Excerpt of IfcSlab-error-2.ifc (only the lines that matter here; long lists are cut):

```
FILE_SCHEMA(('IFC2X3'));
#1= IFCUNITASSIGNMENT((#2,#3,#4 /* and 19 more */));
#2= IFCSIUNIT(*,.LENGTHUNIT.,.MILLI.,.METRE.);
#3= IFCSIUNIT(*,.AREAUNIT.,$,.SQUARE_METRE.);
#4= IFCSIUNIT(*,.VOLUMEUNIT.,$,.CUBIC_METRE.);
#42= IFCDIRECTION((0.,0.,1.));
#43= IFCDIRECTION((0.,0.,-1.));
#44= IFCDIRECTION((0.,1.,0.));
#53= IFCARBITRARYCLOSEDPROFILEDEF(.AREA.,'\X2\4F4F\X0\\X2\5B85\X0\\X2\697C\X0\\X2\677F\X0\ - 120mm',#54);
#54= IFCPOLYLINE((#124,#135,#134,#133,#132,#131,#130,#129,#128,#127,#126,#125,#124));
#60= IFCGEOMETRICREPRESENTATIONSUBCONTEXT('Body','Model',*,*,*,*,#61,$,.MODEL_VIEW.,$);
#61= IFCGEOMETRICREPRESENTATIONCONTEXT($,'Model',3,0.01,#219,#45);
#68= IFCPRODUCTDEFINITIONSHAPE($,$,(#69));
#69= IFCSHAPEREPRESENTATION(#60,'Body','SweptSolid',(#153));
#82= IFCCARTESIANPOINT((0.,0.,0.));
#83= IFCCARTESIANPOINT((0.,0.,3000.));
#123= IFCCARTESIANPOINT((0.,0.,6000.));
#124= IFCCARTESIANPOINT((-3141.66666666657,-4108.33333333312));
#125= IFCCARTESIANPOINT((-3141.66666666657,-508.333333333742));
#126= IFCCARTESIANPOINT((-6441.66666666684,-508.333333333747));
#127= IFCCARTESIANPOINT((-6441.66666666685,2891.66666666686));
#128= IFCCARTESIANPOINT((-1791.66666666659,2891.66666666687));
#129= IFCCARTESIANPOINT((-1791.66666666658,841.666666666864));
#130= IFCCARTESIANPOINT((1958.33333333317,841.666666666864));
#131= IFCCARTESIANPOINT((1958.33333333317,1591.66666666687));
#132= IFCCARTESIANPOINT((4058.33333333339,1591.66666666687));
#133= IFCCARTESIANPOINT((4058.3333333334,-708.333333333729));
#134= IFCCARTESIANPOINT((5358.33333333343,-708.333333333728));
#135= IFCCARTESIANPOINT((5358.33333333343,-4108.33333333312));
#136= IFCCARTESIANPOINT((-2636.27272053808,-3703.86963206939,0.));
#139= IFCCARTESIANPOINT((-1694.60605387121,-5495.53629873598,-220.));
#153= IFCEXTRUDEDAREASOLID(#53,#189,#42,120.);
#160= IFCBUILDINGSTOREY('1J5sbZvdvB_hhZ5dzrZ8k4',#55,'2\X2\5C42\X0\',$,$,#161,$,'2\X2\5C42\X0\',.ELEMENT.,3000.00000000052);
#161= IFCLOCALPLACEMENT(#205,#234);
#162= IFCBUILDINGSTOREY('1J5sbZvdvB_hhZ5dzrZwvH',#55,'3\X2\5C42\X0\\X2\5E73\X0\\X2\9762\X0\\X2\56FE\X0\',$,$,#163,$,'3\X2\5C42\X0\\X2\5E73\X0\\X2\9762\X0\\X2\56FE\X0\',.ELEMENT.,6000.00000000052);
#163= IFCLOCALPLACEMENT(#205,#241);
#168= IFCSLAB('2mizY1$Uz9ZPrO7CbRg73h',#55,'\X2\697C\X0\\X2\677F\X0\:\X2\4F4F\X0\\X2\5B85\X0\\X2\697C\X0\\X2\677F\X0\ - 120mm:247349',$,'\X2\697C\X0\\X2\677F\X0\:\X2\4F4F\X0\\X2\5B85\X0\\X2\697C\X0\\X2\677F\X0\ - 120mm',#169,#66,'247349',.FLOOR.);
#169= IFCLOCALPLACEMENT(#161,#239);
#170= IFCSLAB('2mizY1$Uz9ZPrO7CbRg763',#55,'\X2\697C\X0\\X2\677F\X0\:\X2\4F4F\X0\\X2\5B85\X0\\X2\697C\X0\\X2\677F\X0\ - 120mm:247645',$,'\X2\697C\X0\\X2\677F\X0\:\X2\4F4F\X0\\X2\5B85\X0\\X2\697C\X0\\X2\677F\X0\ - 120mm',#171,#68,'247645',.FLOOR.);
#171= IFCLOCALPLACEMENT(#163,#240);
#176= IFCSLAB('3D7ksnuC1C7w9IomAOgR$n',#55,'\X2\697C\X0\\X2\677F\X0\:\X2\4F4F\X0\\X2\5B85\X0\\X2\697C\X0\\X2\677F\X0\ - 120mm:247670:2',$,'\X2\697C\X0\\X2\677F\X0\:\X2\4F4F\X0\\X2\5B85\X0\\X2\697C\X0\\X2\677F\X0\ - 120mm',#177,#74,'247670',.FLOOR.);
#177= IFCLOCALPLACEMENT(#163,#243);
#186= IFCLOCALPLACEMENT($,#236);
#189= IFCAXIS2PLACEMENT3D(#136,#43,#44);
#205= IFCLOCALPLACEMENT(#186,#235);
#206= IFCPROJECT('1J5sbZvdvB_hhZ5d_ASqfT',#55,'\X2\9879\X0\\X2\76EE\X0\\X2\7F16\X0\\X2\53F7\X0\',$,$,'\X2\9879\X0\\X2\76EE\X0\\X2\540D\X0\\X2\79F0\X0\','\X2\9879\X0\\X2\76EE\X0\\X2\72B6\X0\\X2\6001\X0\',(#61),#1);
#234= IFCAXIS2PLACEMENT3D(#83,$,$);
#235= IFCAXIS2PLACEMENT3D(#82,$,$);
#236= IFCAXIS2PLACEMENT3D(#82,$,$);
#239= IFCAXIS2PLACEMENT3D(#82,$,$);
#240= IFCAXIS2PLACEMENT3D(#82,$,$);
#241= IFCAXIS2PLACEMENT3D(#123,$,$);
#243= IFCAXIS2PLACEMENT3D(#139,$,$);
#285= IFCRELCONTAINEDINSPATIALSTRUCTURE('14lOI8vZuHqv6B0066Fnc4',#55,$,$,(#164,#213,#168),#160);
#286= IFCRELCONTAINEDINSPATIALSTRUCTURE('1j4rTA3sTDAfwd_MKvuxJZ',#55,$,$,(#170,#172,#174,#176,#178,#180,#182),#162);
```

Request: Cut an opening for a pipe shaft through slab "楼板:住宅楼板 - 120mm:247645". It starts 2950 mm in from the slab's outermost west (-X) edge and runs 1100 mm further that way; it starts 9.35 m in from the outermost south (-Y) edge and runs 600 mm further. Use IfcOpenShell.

```python
import numpy as np
import ifcopenshell
import ifcopenshell.api.feature
import ifcopenshell.api.geometry
import ifcopenshell.api.root
import ifcopenshell.geom
import ifcopenshell.util.placement
import ifcopenshell.util.representation
import ifcopenshell.util.shape
import ifcopenshell.util.unit

model = ifcopenshell.open("IfcSlab-error-2.ifc")
unit_scale = ifcopenshell.util.unit.calculate_unit_scale(model)
settings = ifcopenshell.geom.settings()


def volume(element):
    """Net volume in cubic metres, openings subtracted."""
    shape = ifcopenshell.geom.create_shape(settings, element)
    return ifcopenshell.util.shape.get_volume(shape.geometry)


slab = model.by_guid("2mizY1$Uz9ZPrO7CbRg763")
before = volume(slab)

# Extent in the slab's own axes, in metres. The edges named are its -X and -Y sides.
slab_shape = ifcopenshell.geom.create_shape(settings, slab)
vertices = ifcopenshell.util.shape.get_vertices(slab_shape.geometry)
x_min, y_min, bottom = vertices.min(axis=0)
top = vertices[:, 2].max()

opening = ifcopenshell.api.root.create_entity(model, ifc_class="IfcOpeningElement", name="Pipe shaft opening")
context = ifcopenshell.util.representation.get_context(model, "Model", "Body", "MODEL_VIEW")
width, depth = 1.1, 0.6
outline = [(0.0, 0.0), (width, 0.0), (width, depth), (0.0, depth), (0.0, 0.0)]
# Overshoot both faces by 50 mm so the cut is clean.
shape = ifcopenshell.api.geometry.add_slab_representation(
    model, context=context, depth=top - bottom + 0.1, polyline=outline
)
ifcopenshell.api.geometry.assign_representation(model, product=opening, representation=shape)

matrix = ifcopenshell.util.placement.get_local_placement(slab.ObjectPlacement)
matrix[:, 3] = matrix @ np.append(np.array([x_min + 2.95, y_min + 9.35, bottom - 0.05]) / unit_scale, 1.0)
ifcopenshell.api.geometry.edit_object_placement(model, product=opening, matrix=matrix, is_si=False)
ifcopenshell.api.feature.add_feature(model, feature=opening, element=slab)

after = volume(slab)

print(f"slab volume {before:.3f} -> {after:.3f} m3")

model.write("IfcSlab-error-2_v2.ifc")
```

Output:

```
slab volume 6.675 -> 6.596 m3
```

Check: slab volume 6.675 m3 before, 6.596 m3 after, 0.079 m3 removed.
